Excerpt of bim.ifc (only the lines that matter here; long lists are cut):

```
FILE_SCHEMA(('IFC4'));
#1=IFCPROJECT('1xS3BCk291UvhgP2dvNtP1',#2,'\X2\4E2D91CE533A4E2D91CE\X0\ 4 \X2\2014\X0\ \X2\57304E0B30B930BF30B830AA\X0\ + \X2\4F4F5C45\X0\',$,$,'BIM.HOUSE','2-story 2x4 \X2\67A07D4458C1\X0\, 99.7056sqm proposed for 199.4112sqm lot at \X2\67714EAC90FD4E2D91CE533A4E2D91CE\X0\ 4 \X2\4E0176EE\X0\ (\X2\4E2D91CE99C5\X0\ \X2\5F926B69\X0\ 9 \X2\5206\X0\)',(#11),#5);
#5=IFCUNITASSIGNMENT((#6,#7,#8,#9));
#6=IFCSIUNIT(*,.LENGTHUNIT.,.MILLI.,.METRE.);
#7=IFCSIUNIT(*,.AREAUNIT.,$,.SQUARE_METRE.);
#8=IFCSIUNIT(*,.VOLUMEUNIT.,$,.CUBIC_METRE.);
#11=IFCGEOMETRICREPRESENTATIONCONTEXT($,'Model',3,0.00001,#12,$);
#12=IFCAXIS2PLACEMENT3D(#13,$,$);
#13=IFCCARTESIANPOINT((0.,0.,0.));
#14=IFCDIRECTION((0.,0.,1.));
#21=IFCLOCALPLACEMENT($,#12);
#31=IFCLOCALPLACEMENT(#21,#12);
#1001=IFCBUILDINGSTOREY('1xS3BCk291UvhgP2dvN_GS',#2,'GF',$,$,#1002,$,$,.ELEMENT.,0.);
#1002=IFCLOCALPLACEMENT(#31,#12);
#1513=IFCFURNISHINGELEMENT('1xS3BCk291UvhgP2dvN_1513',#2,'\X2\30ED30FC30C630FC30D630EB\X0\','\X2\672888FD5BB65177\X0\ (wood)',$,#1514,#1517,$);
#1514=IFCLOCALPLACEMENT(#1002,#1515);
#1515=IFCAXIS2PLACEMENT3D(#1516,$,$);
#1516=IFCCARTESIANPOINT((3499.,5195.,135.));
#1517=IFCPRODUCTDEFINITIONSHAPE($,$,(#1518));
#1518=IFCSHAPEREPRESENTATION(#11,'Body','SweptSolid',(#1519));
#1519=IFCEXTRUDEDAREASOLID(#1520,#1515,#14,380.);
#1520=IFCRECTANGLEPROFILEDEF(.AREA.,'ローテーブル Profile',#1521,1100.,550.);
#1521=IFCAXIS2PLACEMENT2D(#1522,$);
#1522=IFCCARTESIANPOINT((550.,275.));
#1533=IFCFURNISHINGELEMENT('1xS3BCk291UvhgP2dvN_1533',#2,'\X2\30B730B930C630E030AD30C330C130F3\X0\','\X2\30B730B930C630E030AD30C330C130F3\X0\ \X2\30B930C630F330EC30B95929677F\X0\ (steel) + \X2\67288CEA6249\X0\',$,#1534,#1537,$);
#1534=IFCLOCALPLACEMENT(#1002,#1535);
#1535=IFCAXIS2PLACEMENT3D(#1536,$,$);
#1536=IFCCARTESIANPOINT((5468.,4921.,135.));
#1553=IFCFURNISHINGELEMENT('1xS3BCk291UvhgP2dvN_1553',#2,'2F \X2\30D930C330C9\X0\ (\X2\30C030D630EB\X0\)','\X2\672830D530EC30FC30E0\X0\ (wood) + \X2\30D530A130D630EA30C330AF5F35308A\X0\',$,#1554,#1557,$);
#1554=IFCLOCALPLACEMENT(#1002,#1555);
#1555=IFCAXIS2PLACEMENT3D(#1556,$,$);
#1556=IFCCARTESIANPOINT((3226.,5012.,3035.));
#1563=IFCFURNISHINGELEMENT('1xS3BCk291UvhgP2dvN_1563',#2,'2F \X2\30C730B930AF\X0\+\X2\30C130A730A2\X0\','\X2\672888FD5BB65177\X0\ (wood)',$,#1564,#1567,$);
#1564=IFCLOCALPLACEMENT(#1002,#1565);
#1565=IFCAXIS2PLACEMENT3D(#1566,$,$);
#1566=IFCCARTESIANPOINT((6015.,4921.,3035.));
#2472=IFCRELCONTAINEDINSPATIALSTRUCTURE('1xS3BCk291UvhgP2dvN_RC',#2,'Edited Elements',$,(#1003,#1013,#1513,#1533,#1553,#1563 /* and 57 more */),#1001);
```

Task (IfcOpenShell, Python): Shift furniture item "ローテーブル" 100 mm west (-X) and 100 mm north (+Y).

```python
import ifcopenshell
import ifcopenshell.api.geometry
import ifcopenshell.util.placement
import ifcopenshell.util.unit

model = ifcopenshell.open("bim.ifc")
unit_scale = ifcopenshell.util.unit.calculate_unit_scale(model)

item = model.by_guid("1xS3BCk291UvhgP2dvN_1513")
matrix = ifcopenshell.util.placement.get_local_placement(item.ObjectPlacement)
matrix[0, 3] -= 0.1 / unit_scale
matrix[1, 3] += 0.1 / unit_scale
ifcopenshell.api.geometry.edit_object_placement(model, product=item, matrix=matrix, is_si=False)

print(ifcopenshell.util.placement.get_local_placement(item.ObjectPlacement).round(3) + 0.0)

model.write("bim_edited.ifc")
```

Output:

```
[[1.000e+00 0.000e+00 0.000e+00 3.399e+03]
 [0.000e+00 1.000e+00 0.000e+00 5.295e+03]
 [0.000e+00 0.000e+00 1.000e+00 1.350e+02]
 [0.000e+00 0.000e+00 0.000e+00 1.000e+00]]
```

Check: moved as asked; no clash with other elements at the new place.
